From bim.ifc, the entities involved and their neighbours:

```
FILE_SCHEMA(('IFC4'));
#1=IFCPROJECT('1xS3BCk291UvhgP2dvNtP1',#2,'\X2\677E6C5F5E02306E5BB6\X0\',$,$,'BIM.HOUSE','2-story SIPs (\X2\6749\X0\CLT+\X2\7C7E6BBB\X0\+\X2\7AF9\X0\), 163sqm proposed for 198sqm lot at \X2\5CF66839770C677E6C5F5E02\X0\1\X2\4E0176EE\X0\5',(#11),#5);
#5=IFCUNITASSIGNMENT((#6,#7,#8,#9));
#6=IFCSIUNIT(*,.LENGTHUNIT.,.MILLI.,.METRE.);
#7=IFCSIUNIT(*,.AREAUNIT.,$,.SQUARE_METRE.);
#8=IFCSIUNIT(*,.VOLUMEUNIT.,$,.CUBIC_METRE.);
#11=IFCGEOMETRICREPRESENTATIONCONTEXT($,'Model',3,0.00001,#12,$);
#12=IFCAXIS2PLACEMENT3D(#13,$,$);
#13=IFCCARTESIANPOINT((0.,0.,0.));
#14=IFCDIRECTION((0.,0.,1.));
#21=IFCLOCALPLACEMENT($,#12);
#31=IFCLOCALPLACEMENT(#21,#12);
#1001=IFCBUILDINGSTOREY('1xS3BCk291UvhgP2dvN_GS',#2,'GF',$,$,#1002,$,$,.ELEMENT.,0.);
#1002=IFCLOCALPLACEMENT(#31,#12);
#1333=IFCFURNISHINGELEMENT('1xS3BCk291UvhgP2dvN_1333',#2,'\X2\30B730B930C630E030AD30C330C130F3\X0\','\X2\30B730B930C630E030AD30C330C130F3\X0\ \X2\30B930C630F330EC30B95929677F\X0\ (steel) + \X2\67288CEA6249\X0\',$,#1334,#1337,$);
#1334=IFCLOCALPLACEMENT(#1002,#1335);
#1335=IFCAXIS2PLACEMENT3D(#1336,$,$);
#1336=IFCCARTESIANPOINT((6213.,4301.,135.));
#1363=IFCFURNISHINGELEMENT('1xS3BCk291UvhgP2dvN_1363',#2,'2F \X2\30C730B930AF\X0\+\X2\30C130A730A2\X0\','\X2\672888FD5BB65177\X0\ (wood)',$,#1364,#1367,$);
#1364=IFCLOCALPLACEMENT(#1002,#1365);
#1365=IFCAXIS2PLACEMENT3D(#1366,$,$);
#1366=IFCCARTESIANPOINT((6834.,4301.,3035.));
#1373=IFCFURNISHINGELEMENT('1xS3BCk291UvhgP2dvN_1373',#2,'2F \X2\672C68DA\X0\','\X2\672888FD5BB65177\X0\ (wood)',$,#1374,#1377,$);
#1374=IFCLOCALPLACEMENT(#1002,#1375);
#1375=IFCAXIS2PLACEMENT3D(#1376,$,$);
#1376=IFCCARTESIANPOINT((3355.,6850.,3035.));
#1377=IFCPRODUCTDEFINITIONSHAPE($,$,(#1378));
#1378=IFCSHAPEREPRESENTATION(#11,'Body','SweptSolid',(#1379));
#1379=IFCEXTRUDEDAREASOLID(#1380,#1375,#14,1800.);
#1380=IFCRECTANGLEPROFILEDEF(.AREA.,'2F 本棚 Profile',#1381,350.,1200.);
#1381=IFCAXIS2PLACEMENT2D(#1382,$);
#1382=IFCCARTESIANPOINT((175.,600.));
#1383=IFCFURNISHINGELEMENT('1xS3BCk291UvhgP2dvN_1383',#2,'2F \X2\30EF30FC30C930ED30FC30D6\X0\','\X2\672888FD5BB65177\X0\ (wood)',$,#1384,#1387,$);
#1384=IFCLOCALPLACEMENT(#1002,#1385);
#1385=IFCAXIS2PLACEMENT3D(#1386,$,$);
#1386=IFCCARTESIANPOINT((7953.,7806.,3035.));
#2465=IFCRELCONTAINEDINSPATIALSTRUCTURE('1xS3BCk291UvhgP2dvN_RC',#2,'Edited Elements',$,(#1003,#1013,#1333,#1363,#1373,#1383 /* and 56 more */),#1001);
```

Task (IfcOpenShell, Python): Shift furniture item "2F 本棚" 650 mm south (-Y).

```python
import ifcopenshell
import ifcopenshell.api.geometry
import ifcopenshell.util.placement
import ifcopenshell.util.unit

model = ifcopenshell.open("bim.ifc")
unit_scale = ifcopenshell.util.unit.calculate_unit_scale(model)

item = model.by_guid("1xS3BCk291UvhgP2dvN_1373")
matrix = ifcopenshell.util.placement.get_local_placement(item.ObjectPlacement)
matrix[1, 3] -= 0.65 / unit_scale
ifcopenshell.api.geometry.edit_object_placement(model, product=item, matrix=matrix, is_si=False)

print(ifcopenshell.util.placement.get_local_placement(item.ObjectPlacement).round(3) + 0.0)

model.write("bim_rev.ifc")
```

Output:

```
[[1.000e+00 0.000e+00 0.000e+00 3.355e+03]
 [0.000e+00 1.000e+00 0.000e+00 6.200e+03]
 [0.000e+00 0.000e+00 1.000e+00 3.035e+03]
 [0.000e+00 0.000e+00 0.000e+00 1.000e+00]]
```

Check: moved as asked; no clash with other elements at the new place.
